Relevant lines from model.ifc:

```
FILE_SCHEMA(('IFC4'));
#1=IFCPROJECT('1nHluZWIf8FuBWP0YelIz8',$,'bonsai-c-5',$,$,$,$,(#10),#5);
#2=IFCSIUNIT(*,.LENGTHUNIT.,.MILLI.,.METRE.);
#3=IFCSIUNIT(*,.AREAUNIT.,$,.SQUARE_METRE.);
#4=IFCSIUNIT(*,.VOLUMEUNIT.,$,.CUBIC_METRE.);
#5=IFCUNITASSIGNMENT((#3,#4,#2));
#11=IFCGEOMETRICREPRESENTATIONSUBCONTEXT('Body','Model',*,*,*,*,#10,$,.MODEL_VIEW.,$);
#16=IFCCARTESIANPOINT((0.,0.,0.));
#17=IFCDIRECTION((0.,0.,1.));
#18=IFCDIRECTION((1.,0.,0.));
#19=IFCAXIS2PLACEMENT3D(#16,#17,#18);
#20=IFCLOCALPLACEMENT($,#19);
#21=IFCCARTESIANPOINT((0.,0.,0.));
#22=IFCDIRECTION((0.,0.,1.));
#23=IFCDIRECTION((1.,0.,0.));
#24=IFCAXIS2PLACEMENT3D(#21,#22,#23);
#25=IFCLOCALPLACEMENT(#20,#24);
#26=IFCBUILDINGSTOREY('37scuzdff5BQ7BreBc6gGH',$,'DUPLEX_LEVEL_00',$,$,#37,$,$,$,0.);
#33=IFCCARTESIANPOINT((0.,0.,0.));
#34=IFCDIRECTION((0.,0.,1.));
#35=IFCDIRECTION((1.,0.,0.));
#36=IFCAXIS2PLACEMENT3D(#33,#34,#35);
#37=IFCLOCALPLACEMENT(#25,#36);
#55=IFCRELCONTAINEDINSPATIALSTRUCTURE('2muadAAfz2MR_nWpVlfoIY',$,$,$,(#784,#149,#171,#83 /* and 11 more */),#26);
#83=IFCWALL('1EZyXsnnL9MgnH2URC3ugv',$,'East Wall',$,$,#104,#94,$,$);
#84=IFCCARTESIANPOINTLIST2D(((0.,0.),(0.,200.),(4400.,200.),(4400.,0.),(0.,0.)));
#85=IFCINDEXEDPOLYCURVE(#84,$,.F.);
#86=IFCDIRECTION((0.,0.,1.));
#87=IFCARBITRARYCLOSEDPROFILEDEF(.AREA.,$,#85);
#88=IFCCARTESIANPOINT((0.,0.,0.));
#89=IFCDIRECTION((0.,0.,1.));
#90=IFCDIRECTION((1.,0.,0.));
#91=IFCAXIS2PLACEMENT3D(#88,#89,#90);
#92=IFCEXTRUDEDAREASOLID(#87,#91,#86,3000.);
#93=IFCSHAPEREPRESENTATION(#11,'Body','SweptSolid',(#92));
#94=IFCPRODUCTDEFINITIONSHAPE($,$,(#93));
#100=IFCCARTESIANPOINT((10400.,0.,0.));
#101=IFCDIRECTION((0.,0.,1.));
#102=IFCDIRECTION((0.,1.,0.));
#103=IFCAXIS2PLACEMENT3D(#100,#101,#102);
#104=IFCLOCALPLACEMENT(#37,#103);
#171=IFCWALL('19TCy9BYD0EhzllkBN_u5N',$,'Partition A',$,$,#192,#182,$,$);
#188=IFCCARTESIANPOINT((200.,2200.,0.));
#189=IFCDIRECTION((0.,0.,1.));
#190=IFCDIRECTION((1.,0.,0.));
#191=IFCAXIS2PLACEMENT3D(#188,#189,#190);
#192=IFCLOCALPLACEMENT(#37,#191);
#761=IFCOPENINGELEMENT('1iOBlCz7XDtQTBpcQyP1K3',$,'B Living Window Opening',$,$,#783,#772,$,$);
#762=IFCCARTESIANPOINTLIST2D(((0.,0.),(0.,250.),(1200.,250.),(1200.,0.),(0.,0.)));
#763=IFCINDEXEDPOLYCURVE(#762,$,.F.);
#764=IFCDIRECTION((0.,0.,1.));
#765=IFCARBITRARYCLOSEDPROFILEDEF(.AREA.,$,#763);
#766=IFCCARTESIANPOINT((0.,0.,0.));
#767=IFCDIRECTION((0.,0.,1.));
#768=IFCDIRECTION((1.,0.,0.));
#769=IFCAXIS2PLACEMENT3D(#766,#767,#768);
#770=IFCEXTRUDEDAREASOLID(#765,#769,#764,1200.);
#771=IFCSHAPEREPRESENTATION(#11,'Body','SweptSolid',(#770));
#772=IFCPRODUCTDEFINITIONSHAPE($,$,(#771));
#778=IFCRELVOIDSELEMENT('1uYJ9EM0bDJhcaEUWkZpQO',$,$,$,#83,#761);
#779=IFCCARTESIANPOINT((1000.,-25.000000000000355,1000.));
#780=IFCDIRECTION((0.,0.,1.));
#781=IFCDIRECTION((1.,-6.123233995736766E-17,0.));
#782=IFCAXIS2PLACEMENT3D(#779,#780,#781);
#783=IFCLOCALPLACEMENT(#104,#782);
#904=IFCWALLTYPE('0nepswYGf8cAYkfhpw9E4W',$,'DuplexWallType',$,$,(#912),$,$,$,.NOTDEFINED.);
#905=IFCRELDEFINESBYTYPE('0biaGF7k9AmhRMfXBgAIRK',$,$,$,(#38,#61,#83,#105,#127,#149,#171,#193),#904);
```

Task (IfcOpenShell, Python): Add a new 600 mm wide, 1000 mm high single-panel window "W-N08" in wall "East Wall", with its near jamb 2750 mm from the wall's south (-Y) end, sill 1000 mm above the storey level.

```python
import numpy as np
import ifcopenshell
import ifcopenshell.api.feature
import ifcopenshell.api.geometry
import ifcopenshell.api.root
import ifcopenshell.api.spatial
import ifcopenshell.geom
import ifcopenshell.util.element
import ifcopenshell.util.placement
import ifcopenshell.util.representation
import ifcopenshell.util.shape
import ifcopenshell.util.unit

model = ifcopenshell.open("model.ifc")
unit_scale = ifcopenshell.util.unit.calculate_unit_scale(model)
settings = ifcopenshell.geom.settings()


def volume(element):
    """Net volume in cubic metres, openings subtracted."""
    shape = ifcopenshell.geom.create_shape(settings, element)
    return ifcopenshell.util.shape.get_volume(shape.geometry)


wall = model.by_guid("1EZyXsnnL9MgnH2URC3ugv")
storey = ifcopenshell.util.element.get_container(wall, ifc_class="IfcBuildingStorey")
context = ifcopenshell.util.representation.get_context(model, "Model", "Body", "MODEL_VIEW")
before = volume(wall)

width, height, from_end, sill = 0.6, 1, 2.75, 1  # metres

# The wall runs along its own X axis, and the end named is its -X end.
wall_shape = ifcopenshell.geom.create_shape(settings, wall)
x, y, z = ifcopenshell.util.shape.get_vertices(wall_shape.geometry).T
start = x.min() + from_end
face, thickness = float(y.min()), float(y.max() - y.min())
wall_matrix = ifcopenshell.util.placement.get_local_placement(wall.ObjectPlacement)
level = ifcopenshell.util.placement.get_local_placement(storey.ObjectPlacement)[2, 3]


def in_wall(x, y):
    """Placement at x, y metres in the wall's axes, at sill height."""
    matrix = wall_matrix.copy()
    matrix[:, 3] = wall_matrix @ np.array([x / unit_scale, y / unit_scale, 0.0, 1.0])
    matrix[2, 3] = level + sill / unit_scale
    return matrix


# Opening: a box that overshoots both wall faces by 50 mm.
opening = ifcopenshell.api.root.create_entity(model, ifc_class="IfcOpeningElement", predefined_type="OPENING")
box = ifcopenshell.api.geometry.add_wall_representation(
    model, context=context, length=width, height=height, thickness=thickness + 0.1
)
ifcopenshell.api.geometry.assign_representation(model, product=opening, representation=box)
ifcopenshell.api.geometry.edit_object_placement(model, product=opening, matrix=in_wall(start, face - 0.05), is_si=False)
ifcopenshell.api.feature.add_feature(model, feature=opening, element=wall)

window = ifcopenshell.api.root.create_entity(model, ifc_class="IfcWindow", name="W-N08", predefined_type="WINDOW")
window.OverallWidth, window.OverallHeight = width / unit_scale, height / unit_scale
window.PartitioningType = "SINGLE_PANEL"
body = ifcopenshell.api.geometry.add_window_representation(
    model,
    context=context,
    overall_width=window.OverallWidth,
    overall_height=window.OverallHeight,
    partition_type="SINGLE_PANEL",
)
ifcopenshell.api.geometry.assign_representation(model, product=window, representation=body)
ifcopenshell.api.spatial.assign_container(model, products=[window], relating_structure=storey)
ifcopenshell.api.feature.add_filling(model, opening=opening, element=window)

# Centre the window in the wall's thickness.
ifcopenshell.api.geometry.edit_object_placement(model, product=window, matrix=in_wall(start, face), is_si=False)
window_shape = ifcopenshell.geom.create_shape(settings, window)
depth = ifcopenshell.util.shape.get_vertices(window_shape.geometry)[:, 1]
offset = face + thickness / 2 - (depth.min() + depth.max()) / 2
ifcopenshell.api.geometry.edit_object_placement(model, product=window, matrix=in_wall(start, offset), is_si=False)

after = volume(wall)

print(f"wall volume {before:.3f} -> {after:.3f} m3")

model.write("model_v2.ifc")
```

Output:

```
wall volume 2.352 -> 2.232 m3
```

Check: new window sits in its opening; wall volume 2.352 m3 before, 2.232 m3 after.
